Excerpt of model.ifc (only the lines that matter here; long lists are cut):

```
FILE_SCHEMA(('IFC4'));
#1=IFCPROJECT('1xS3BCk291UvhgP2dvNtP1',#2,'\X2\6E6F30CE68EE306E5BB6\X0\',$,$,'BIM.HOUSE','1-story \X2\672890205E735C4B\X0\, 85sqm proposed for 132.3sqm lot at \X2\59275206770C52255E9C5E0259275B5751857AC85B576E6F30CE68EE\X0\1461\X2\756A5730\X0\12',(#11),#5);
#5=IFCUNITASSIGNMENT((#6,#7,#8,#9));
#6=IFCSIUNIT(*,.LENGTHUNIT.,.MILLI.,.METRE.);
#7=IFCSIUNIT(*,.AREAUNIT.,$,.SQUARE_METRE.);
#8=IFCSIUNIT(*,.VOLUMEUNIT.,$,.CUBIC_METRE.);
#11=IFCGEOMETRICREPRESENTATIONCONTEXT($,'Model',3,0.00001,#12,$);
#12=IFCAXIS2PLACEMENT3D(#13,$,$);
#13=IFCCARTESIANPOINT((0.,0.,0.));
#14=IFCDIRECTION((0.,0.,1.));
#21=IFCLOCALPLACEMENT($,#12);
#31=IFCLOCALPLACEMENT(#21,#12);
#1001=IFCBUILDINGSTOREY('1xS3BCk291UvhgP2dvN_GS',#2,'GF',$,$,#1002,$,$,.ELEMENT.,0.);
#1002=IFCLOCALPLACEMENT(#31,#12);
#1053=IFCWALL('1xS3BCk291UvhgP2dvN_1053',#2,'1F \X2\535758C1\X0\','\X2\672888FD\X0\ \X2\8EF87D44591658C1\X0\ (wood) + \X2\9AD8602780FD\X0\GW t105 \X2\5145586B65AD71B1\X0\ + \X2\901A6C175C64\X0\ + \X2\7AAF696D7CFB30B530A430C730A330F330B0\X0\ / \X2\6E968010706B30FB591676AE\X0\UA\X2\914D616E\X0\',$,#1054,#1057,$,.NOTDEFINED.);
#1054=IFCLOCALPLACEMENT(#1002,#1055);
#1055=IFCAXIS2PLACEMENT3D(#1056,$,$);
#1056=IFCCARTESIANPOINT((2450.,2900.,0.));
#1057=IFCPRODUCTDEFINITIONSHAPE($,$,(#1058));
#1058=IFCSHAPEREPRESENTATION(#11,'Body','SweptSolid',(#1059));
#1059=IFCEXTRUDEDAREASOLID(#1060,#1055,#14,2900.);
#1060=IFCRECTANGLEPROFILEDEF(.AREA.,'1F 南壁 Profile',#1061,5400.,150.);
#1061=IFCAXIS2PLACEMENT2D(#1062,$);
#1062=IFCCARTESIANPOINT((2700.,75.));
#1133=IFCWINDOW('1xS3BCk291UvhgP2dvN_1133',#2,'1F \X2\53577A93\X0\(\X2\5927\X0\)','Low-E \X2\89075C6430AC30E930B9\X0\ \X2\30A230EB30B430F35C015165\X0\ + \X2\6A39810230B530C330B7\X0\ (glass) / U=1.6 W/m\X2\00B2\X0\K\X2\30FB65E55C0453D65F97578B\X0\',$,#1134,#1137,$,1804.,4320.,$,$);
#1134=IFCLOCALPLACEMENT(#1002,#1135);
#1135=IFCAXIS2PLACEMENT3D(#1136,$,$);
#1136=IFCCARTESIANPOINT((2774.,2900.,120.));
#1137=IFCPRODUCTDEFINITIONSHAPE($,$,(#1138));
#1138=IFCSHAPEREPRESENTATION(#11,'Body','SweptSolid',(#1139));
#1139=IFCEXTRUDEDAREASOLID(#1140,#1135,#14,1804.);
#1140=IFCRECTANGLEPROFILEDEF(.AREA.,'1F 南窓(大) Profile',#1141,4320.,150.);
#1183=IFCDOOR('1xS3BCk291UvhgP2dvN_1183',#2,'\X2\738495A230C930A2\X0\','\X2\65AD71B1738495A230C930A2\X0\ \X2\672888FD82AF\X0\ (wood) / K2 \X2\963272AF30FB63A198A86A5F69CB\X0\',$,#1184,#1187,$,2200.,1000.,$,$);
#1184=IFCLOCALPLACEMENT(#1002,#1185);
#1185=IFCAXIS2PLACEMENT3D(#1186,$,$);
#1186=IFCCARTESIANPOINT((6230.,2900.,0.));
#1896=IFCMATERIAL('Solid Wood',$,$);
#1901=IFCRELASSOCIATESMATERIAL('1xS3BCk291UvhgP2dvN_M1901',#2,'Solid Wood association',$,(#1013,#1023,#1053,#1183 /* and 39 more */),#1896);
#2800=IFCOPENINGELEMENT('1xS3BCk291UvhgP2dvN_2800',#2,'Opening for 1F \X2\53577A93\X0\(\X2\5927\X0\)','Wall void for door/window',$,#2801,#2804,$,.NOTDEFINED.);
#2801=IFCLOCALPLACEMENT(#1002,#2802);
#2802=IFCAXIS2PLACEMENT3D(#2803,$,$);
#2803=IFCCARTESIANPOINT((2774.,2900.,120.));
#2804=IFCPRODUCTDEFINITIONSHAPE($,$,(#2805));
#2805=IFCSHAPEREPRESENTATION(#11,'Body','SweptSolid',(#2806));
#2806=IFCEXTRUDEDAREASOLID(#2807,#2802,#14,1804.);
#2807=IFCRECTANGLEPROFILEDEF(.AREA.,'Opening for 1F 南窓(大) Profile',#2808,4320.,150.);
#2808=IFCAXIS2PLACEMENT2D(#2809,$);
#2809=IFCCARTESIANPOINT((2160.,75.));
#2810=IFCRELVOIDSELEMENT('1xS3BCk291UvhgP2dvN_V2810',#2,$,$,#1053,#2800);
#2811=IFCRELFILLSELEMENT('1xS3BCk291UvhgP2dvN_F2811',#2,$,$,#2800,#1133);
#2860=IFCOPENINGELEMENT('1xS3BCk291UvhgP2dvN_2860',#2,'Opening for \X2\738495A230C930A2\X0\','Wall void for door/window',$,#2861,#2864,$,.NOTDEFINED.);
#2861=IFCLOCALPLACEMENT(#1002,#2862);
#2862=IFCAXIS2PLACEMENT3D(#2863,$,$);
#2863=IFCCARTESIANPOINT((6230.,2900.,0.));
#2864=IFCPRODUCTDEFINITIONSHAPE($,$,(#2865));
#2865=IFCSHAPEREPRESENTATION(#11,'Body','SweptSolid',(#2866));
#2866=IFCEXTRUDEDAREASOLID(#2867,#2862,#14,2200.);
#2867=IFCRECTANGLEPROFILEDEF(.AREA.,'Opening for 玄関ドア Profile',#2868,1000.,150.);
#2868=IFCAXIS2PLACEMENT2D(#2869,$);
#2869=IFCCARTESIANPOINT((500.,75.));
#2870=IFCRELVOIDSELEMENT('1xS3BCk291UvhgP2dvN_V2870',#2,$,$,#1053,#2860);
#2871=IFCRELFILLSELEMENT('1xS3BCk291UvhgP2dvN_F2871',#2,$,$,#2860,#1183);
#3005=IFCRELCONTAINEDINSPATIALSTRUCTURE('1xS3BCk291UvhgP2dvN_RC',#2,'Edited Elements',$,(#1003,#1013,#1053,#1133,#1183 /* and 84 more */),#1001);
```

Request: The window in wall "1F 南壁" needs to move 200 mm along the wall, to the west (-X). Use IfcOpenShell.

```python
import ifcopenshell
import ifcopenshell.api.geometry
import ifcopenshell.util.placement
import ifcopenshell.util.unit

model = ifcopenshell.open("model.ifc")
unit_scale = ifcopenshell.util.unit.calculate_unit_scale(model)

window = model.by_id(1133)
opening = window.FillsVoids[0].RelatingOpeningElement
wall = opening.VoidsElements[0].RelatingBuildingElement

wall_matrix = ifcopenshell.util.placement.get_local_placement(wall.ObjectPlacement)
shift = wall_matrix[:3, 0] * -0.2 / unit_scale
before = ifcopenshell.util.placement.get_local_placement(window.ObjectPlacement)[:3, 3].copy()

# The window is not placed relative to its opening, so move both.
for product in (opening, window):
    matrix = ifcopenshell.util.placement.get_local_placement(product.ObjectPlacement)
    matrix[:3, 3] += shift
    ifcopenshell.api.geometry.edit_object_placement(model, product=product, matrix=matrix, is_si=False)

after = ifcopenshell.util.placement.get_local_placement(window.ObjectPlacement)[:3, 3]
print("window moved by", (after - before).round(3) + 0.0)

model.write("model_edited.ifc")
```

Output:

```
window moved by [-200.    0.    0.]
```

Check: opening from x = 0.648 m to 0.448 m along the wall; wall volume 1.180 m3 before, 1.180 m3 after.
